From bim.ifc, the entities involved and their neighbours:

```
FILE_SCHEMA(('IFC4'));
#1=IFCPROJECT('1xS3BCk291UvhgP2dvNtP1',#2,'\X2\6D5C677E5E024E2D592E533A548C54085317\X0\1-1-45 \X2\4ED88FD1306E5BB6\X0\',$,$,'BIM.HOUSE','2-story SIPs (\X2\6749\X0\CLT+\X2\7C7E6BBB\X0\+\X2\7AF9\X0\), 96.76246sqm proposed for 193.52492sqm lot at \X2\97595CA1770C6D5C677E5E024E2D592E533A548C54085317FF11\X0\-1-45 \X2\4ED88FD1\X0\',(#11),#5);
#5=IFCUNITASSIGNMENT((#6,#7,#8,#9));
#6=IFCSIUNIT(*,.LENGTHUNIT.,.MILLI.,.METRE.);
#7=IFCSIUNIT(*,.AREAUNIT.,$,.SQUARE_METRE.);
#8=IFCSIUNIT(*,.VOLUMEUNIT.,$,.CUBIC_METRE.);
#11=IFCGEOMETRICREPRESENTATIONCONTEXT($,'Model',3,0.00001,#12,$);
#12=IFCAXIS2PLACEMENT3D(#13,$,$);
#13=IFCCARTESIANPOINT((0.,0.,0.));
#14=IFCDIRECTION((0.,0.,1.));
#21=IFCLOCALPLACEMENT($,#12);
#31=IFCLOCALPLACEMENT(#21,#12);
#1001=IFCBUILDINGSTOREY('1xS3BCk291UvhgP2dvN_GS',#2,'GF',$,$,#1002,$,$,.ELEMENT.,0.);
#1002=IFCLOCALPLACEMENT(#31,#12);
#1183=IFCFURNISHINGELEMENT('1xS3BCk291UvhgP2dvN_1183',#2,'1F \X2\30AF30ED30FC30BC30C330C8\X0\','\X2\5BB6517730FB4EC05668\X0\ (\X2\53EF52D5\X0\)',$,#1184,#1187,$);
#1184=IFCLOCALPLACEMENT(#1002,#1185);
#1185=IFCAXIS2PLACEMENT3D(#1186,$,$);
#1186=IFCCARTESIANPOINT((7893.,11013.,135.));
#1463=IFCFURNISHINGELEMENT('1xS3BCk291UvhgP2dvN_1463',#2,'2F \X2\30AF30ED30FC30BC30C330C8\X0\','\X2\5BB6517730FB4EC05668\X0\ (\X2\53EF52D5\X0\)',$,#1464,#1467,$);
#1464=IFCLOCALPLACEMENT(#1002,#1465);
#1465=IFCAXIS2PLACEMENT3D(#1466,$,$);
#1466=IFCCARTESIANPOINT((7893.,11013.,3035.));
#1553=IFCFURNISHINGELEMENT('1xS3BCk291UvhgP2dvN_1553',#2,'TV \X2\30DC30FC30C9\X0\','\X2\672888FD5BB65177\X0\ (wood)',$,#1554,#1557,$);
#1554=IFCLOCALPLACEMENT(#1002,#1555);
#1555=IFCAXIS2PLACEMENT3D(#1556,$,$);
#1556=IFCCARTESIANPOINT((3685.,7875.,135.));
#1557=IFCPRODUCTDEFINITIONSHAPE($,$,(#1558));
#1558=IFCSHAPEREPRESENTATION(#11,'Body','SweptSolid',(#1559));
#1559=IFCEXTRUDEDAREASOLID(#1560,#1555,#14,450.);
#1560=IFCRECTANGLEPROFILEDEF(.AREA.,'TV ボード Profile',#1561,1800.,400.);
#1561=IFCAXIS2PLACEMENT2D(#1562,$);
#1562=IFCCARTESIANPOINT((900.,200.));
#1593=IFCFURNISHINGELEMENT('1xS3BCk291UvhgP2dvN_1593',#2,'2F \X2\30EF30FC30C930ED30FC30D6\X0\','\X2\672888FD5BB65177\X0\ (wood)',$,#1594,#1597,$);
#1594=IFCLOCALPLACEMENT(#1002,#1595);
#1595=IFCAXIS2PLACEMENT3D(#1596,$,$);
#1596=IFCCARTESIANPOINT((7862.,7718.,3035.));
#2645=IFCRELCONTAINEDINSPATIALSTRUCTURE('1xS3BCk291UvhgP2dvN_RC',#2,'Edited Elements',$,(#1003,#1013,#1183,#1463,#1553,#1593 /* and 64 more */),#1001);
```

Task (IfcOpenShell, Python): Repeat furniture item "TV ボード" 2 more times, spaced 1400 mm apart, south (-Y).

```python
import numpy as np
import ifcopenshell
import ifcopenshell.api.geometry
import ifcopenshell.api.root
import ifcopenshell.util.element
import ifcopenshell.util.placement
import ifcopenshell.util.unit

model = ifcopenshell.open("bim.ifc")
unit_scale = ifcopenshell.util.unit.calculate_unit_scale(model)


def reuse_history(source, copy):
    """copy_class also copies each property set's owner history, people and application; keep the originals."""
    for rel in copy.IsDefinedBy:
        if rel.is_a("IfcRelDefinesByProperties") and (history := rel.RelatingPropertyDefinition.OwnerHistory):
            rel.RelatingPropertyDefinition.OwnerHistory = source.OwnerHistory
            ifcopenshell.util.element.remove_deep2(model, history)


source = model.by_guid("1xS3BCk291UvhgP2dvN_1553")
base = ifcopenshell.util.placement.get_local_placement(source.ObjectPlacement)
step = np.array([0.0, -1.0, 0.0]) * 1.4 / unit_scale

for i in range(1, 3):
    copy = ifcopenshell.api.root.copy_class(model, product=source)
    copy.Representation = ifcopenshell.util.element.copy_deep(
        model, source.Representation, exclude=["IfcGeometricRepresentationContext", "IfcRepresentationMap"]
    )
    reuse_history(source, copy)
    matrix = base.copy()
    matrix[:3, 3] += i * step
    print("added at", matrix[:3, 3].round(3) + 0.0)
    ifcopenshell.api.geometry.edit_object_placement(model, product=copy, matrix=matrix, is_si=False)

model.write("bim_updated.ifc")
```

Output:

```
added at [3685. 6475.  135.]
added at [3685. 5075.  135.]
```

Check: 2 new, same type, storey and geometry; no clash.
